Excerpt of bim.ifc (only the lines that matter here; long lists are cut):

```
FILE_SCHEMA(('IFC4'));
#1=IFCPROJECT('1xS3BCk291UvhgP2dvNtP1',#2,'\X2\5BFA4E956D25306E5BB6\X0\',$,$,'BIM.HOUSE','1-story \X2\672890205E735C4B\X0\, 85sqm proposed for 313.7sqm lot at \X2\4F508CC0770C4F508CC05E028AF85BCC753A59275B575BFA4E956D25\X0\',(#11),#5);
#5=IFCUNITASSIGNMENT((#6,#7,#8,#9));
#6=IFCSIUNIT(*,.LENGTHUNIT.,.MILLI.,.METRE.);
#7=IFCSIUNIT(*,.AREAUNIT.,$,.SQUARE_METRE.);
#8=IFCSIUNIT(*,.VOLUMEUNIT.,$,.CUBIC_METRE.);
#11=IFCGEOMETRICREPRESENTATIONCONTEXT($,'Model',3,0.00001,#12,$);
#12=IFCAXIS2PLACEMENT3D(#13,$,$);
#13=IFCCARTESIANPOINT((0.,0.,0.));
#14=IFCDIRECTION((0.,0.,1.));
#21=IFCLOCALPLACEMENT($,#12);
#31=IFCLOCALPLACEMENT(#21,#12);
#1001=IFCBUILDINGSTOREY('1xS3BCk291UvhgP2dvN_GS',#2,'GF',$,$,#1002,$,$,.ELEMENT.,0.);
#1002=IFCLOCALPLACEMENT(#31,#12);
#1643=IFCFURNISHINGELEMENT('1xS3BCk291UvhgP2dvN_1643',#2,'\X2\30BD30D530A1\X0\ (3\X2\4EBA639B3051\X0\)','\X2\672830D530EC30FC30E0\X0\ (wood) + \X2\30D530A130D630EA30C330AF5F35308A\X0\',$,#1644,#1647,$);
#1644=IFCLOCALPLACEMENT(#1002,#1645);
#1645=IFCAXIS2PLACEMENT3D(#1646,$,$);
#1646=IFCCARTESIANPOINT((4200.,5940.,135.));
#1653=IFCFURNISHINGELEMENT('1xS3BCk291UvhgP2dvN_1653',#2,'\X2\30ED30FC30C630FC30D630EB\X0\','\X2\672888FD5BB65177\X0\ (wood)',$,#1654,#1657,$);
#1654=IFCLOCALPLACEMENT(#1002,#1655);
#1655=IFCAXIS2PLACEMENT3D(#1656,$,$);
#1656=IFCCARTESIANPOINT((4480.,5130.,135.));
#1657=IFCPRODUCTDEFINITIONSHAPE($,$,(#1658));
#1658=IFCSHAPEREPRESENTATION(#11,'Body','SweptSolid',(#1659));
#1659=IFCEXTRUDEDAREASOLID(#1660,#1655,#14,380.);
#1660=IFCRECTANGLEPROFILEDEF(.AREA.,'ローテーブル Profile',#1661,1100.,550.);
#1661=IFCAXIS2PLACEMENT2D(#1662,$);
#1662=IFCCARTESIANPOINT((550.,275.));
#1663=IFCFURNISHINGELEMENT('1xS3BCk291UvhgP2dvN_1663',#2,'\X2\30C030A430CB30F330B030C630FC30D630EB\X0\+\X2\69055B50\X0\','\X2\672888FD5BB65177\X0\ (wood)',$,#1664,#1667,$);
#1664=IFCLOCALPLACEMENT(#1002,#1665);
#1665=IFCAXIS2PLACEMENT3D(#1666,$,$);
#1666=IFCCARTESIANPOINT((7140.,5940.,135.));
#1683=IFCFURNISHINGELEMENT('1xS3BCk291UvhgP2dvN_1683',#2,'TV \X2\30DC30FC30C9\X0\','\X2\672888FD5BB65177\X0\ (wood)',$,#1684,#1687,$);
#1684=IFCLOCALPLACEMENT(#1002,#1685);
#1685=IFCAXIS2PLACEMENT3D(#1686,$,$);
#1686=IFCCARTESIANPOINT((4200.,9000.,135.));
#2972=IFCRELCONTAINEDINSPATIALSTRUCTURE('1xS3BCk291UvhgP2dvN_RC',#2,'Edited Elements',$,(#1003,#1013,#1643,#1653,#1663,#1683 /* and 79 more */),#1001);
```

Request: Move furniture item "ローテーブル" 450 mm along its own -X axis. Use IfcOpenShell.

```python
import ifcopenshell
import ifcopenshell.api.geometry
import ifcopenshell.util.placement
import ifcopenshell.util.unit

model = ifcopenshell.open("bim.ifc")
unit_scale = ifcopenshell.util.unit.calculate_unit_scale(model)

item = model.by_guid("1xS3BCk291UvhgP2dvN_1653")
matrix = ifcopenshell.util.placement.get_local_placement(item.ObjectPlacement)
matrix[:3, 3] -= matrix[:3, 0] * 0.45 / unit_scale
ifcopenshell.api.geometry.edit_object_placement(model, product=item, matrix=matrix, is_si=False)

print(ifcopenshell.util.placement.get_local_placement(item.ObjectPlacement).round(3) + 0.0)

model.write("bim-out.ifc")
```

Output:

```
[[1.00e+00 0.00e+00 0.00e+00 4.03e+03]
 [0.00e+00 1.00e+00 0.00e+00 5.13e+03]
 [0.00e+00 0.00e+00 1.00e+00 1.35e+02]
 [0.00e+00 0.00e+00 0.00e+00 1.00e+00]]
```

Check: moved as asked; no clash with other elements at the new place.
